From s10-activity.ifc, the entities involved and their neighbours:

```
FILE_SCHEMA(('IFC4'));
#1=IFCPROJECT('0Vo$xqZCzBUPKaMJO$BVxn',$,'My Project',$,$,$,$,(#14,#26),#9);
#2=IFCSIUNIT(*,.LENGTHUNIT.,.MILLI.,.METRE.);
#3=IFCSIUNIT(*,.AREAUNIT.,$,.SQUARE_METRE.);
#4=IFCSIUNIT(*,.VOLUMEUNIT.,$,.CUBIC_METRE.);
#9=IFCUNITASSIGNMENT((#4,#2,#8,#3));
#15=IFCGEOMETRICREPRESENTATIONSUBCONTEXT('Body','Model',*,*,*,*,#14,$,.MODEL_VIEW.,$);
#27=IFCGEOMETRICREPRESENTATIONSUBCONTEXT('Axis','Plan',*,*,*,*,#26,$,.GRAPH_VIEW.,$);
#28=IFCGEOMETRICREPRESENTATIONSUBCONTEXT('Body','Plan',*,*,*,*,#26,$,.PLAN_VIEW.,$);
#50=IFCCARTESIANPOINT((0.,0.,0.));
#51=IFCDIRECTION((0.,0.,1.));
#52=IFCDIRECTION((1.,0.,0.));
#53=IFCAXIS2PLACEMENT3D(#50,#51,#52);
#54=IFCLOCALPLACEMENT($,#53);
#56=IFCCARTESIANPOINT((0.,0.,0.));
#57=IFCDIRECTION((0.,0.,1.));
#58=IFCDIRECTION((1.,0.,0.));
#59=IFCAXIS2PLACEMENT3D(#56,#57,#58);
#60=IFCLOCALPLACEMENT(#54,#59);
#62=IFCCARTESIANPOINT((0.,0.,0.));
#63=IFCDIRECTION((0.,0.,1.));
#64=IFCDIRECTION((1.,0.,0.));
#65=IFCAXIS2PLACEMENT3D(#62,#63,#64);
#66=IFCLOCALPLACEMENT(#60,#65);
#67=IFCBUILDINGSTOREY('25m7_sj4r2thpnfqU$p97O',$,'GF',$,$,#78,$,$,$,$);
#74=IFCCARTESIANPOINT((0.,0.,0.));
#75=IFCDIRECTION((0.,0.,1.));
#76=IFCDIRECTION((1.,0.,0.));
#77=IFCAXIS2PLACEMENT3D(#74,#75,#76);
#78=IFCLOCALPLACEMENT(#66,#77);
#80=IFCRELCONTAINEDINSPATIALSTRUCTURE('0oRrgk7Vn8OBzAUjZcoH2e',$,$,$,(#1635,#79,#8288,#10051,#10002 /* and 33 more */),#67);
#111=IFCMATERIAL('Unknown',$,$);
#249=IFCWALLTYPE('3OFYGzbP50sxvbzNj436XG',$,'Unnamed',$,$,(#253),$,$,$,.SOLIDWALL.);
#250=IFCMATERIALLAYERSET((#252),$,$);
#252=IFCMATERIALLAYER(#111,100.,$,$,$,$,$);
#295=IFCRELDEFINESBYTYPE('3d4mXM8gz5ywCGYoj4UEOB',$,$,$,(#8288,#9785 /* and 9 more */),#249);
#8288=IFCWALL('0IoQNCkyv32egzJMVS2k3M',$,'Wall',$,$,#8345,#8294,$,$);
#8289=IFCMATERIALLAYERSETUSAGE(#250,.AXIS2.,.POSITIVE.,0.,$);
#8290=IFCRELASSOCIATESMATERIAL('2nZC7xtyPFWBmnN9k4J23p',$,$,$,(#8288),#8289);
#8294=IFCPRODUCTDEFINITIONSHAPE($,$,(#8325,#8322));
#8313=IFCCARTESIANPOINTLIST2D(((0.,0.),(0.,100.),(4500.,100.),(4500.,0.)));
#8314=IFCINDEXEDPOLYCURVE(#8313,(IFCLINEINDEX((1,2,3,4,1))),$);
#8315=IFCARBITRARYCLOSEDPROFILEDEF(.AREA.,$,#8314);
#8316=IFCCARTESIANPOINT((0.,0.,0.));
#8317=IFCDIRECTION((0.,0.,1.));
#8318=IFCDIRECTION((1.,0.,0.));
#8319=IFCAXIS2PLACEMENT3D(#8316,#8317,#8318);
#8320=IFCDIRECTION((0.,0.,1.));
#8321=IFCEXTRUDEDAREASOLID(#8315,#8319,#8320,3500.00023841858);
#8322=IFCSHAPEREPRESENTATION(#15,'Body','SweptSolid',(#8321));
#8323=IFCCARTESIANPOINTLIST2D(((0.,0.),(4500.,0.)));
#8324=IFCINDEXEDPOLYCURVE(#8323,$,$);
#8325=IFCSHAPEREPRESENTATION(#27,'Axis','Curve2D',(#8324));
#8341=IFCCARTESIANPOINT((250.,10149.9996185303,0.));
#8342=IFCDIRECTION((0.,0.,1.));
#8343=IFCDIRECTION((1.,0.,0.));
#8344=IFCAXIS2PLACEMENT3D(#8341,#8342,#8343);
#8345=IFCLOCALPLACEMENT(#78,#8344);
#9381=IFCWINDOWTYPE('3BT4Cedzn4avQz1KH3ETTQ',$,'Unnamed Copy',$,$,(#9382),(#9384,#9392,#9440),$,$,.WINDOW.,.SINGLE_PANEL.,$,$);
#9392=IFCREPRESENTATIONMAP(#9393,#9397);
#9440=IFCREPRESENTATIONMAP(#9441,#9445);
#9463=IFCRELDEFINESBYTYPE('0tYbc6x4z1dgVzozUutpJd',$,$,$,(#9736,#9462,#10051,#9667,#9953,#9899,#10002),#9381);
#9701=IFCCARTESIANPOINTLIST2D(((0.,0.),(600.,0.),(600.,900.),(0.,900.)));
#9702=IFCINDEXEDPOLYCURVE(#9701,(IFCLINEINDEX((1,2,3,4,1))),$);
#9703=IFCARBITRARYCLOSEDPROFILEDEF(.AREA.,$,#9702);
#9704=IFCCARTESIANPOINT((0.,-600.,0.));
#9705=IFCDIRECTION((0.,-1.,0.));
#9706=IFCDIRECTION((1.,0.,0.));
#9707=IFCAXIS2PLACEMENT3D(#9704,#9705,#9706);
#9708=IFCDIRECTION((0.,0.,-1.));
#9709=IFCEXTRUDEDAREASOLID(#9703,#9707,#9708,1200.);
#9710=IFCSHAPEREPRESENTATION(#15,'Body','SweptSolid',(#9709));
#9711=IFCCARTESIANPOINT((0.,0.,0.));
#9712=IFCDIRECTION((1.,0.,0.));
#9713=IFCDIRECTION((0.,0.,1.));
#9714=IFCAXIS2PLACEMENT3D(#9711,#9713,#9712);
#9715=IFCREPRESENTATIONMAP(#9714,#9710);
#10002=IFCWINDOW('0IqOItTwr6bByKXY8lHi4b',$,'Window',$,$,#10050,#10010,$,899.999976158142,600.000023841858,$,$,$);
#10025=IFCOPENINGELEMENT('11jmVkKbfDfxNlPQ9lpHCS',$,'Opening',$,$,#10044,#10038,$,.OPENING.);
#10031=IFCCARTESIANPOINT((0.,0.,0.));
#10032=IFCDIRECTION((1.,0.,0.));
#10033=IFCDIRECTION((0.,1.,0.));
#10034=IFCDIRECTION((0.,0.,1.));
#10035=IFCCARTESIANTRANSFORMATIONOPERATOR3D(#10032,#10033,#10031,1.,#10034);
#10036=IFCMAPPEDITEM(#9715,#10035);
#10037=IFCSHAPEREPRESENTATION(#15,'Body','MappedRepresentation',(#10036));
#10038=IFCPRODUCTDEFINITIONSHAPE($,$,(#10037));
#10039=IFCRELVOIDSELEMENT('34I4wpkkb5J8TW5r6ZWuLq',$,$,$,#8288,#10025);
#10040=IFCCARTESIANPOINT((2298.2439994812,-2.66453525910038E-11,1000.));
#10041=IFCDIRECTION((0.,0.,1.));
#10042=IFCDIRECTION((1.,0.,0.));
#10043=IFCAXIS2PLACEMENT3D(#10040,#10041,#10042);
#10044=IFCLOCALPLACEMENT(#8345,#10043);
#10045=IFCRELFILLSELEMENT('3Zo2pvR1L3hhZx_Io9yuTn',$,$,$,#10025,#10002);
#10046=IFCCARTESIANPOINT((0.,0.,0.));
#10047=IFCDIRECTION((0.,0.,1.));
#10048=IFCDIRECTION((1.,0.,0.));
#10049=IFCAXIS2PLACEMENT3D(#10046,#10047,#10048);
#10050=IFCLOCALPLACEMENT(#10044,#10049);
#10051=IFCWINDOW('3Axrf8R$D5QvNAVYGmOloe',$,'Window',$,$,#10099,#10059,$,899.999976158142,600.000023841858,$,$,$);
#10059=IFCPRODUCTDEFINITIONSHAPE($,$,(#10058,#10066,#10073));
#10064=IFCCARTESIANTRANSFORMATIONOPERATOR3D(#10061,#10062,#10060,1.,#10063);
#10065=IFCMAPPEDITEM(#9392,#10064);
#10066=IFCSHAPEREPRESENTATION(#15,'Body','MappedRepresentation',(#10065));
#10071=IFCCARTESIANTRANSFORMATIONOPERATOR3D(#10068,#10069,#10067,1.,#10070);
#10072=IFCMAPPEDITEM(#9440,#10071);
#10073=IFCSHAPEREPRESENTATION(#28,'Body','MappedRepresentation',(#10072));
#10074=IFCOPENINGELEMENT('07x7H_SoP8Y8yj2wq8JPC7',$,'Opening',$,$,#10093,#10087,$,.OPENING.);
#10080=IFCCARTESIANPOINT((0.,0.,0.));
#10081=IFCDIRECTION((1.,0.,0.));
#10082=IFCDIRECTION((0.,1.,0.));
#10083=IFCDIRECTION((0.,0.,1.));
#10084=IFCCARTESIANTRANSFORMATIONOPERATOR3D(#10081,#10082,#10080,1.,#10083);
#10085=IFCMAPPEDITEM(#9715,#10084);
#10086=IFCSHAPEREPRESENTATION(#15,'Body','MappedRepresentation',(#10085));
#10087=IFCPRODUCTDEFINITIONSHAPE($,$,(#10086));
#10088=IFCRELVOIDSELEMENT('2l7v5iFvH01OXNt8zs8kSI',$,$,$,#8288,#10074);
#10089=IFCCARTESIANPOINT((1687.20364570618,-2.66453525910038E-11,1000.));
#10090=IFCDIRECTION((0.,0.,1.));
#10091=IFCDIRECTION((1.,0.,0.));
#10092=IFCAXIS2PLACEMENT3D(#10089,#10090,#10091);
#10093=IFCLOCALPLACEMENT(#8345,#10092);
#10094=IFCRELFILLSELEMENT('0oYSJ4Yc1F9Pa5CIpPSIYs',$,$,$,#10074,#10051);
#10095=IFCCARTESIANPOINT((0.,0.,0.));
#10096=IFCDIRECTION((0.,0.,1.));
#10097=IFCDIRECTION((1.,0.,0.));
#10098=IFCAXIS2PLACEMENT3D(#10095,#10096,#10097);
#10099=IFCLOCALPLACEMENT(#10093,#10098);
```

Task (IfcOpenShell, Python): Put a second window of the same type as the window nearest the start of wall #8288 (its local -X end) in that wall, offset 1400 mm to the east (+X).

```python
import ifcopenshell
import ifcopenshell.api.feature
import ifcopenshell.api.geometry
import ifcopenshell.api.root
import ifcopenshell.geom
import ifcopenshell.util.element
import ifcopenshell.util.placement
import ifcopenshell.util.shape

model = ifcopenshell.open("s10-activity.ifc")
settings = ifcopenshell.geom.settings()


def volume(element):
    """Net volume in cubic metres, openings subtracted."""
    shape = ifcopenshell.geom.create_shape(settings, element)
    return ifcopenshell.util.shape.get_volume(shape.geometry)


window = model.by_guid("3Axrf8R$D5QvNAVYGmOloe")
opening = window.FillsVoids[0].RelatingOpeningElement
wall = opening.VoidsElements[0].RelatingBuildingElement
before = volume(wall)
shift = ifcopenshell.util.placement.get_local_placement(wall.ObjectPlacement)[:3, 0] * 1400.0

# copy_class copies the void relationship, type, container and properties, but no geometry.
new_opening = ifcopenshell.api.root.copy_class(model, product=opening)
new_opening.Representation = ifcopenshell.util.element.copy_deep(
    model, opening.Representation, exclude=["IfcGeometricRepresentationContext", "IfcRepresentationMap"]
)
new_window = ifcopenshell.api.root.copy_class(model, product=window)
new_window.Representation = ifcopenshell.util.element.copy_deep(
    model, window.Representation, exclude=["IfcGeometricRepresentationContext", "IfcRepresentationMap"]
)
ifcopenshell.api.feature.add_filling(model, opening=new_opening, element=new_window)

for old, new in ((opening, new_opening), (window, new_window)):
    matrix = ifcopenshell.util.placement.get_local_placement(old.ObjectPlacement)
    matrix[:3, 3] += shift
    ifcopenshell.api.geometry.edit_object_placement(model, product=new, matrix=matrix, is_si=False)

after = volume(wall)

print(f"wall volume {before:.3f} -> {after:.3f} m3")

model.write("s10-activity_rev.ifc")
```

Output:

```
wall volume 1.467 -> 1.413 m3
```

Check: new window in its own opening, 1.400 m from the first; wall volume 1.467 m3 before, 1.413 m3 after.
